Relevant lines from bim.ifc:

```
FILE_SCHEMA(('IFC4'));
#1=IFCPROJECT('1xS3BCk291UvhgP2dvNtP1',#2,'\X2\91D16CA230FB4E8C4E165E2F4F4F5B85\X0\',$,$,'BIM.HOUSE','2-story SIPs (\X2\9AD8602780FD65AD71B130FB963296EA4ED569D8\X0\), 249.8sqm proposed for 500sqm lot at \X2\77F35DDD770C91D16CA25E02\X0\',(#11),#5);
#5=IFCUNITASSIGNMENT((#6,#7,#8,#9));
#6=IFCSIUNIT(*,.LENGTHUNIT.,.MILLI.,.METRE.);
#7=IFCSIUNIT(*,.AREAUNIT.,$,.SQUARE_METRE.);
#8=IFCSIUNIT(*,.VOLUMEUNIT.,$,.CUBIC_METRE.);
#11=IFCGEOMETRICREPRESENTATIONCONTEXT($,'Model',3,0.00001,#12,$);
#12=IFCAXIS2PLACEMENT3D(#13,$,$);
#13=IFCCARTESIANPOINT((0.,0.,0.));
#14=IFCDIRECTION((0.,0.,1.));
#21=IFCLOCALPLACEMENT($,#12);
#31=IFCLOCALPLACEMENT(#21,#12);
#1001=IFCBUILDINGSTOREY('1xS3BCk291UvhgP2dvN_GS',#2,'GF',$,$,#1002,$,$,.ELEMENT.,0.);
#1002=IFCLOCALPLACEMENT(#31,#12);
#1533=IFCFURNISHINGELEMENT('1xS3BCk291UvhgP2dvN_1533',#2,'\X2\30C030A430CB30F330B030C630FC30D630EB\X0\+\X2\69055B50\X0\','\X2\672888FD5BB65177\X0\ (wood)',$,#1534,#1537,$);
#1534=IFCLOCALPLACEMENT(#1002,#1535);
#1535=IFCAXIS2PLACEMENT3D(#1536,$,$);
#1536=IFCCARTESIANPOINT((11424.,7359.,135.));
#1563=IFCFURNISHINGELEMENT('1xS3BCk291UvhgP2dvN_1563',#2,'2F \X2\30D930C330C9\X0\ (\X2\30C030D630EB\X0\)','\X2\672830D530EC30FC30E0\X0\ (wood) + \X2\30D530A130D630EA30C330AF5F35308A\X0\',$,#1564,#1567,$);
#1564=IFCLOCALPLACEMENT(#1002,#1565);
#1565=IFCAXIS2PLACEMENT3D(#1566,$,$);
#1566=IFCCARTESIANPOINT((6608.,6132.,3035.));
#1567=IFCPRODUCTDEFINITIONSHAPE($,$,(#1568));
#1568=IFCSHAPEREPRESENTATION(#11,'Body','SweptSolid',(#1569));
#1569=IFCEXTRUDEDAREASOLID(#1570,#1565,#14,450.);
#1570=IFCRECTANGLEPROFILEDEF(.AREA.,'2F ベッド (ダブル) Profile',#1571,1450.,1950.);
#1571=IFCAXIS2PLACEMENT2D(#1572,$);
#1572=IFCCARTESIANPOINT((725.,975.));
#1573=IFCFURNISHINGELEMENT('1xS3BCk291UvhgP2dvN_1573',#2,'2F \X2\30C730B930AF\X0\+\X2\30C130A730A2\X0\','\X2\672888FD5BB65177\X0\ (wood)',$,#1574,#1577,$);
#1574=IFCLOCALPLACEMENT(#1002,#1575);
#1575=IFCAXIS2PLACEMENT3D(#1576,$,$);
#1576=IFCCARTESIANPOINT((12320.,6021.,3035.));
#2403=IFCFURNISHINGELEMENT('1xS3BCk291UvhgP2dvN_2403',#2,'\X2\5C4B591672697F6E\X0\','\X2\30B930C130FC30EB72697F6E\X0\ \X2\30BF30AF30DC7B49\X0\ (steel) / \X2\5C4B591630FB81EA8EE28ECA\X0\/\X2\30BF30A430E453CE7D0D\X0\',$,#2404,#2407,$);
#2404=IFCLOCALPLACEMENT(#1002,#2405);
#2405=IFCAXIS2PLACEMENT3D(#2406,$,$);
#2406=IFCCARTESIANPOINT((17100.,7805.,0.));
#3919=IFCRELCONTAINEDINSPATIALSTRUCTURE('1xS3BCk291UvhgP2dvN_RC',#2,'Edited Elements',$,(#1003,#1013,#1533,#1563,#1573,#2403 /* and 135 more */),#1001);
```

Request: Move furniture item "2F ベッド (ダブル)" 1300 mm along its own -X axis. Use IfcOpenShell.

```python
import ifcopenshell
import ifcopenshell.api.geometry
import ifcopenshell.util.placement

model = ifcopenshell.open("bim.ifc")

item = model.by_guid("1xS3BCk291UvhgP2dvN_1563")
matrix = ifcopenshell.util.placement.get_local_placement(item.ObjectPlacement)
matrix[:3, 3] -= matrix[:3, 0] * 1300.0
ifcopenshell.api.geometry.edit_object_placement(model, product=item, matrix=matrix, is_si=False)

print(ifcopenshell.util.placement.get_local_placement(item.ObjectPlacement).round(3) + 0.0)

model.write("bim_updated.ifc")
```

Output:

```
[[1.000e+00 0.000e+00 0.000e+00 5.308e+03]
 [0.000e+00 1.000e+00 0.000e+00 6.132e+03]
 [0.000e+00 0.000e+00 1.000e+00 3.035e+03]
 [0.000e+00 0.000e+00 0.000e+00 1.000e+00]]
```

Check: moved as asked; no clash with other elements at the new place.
